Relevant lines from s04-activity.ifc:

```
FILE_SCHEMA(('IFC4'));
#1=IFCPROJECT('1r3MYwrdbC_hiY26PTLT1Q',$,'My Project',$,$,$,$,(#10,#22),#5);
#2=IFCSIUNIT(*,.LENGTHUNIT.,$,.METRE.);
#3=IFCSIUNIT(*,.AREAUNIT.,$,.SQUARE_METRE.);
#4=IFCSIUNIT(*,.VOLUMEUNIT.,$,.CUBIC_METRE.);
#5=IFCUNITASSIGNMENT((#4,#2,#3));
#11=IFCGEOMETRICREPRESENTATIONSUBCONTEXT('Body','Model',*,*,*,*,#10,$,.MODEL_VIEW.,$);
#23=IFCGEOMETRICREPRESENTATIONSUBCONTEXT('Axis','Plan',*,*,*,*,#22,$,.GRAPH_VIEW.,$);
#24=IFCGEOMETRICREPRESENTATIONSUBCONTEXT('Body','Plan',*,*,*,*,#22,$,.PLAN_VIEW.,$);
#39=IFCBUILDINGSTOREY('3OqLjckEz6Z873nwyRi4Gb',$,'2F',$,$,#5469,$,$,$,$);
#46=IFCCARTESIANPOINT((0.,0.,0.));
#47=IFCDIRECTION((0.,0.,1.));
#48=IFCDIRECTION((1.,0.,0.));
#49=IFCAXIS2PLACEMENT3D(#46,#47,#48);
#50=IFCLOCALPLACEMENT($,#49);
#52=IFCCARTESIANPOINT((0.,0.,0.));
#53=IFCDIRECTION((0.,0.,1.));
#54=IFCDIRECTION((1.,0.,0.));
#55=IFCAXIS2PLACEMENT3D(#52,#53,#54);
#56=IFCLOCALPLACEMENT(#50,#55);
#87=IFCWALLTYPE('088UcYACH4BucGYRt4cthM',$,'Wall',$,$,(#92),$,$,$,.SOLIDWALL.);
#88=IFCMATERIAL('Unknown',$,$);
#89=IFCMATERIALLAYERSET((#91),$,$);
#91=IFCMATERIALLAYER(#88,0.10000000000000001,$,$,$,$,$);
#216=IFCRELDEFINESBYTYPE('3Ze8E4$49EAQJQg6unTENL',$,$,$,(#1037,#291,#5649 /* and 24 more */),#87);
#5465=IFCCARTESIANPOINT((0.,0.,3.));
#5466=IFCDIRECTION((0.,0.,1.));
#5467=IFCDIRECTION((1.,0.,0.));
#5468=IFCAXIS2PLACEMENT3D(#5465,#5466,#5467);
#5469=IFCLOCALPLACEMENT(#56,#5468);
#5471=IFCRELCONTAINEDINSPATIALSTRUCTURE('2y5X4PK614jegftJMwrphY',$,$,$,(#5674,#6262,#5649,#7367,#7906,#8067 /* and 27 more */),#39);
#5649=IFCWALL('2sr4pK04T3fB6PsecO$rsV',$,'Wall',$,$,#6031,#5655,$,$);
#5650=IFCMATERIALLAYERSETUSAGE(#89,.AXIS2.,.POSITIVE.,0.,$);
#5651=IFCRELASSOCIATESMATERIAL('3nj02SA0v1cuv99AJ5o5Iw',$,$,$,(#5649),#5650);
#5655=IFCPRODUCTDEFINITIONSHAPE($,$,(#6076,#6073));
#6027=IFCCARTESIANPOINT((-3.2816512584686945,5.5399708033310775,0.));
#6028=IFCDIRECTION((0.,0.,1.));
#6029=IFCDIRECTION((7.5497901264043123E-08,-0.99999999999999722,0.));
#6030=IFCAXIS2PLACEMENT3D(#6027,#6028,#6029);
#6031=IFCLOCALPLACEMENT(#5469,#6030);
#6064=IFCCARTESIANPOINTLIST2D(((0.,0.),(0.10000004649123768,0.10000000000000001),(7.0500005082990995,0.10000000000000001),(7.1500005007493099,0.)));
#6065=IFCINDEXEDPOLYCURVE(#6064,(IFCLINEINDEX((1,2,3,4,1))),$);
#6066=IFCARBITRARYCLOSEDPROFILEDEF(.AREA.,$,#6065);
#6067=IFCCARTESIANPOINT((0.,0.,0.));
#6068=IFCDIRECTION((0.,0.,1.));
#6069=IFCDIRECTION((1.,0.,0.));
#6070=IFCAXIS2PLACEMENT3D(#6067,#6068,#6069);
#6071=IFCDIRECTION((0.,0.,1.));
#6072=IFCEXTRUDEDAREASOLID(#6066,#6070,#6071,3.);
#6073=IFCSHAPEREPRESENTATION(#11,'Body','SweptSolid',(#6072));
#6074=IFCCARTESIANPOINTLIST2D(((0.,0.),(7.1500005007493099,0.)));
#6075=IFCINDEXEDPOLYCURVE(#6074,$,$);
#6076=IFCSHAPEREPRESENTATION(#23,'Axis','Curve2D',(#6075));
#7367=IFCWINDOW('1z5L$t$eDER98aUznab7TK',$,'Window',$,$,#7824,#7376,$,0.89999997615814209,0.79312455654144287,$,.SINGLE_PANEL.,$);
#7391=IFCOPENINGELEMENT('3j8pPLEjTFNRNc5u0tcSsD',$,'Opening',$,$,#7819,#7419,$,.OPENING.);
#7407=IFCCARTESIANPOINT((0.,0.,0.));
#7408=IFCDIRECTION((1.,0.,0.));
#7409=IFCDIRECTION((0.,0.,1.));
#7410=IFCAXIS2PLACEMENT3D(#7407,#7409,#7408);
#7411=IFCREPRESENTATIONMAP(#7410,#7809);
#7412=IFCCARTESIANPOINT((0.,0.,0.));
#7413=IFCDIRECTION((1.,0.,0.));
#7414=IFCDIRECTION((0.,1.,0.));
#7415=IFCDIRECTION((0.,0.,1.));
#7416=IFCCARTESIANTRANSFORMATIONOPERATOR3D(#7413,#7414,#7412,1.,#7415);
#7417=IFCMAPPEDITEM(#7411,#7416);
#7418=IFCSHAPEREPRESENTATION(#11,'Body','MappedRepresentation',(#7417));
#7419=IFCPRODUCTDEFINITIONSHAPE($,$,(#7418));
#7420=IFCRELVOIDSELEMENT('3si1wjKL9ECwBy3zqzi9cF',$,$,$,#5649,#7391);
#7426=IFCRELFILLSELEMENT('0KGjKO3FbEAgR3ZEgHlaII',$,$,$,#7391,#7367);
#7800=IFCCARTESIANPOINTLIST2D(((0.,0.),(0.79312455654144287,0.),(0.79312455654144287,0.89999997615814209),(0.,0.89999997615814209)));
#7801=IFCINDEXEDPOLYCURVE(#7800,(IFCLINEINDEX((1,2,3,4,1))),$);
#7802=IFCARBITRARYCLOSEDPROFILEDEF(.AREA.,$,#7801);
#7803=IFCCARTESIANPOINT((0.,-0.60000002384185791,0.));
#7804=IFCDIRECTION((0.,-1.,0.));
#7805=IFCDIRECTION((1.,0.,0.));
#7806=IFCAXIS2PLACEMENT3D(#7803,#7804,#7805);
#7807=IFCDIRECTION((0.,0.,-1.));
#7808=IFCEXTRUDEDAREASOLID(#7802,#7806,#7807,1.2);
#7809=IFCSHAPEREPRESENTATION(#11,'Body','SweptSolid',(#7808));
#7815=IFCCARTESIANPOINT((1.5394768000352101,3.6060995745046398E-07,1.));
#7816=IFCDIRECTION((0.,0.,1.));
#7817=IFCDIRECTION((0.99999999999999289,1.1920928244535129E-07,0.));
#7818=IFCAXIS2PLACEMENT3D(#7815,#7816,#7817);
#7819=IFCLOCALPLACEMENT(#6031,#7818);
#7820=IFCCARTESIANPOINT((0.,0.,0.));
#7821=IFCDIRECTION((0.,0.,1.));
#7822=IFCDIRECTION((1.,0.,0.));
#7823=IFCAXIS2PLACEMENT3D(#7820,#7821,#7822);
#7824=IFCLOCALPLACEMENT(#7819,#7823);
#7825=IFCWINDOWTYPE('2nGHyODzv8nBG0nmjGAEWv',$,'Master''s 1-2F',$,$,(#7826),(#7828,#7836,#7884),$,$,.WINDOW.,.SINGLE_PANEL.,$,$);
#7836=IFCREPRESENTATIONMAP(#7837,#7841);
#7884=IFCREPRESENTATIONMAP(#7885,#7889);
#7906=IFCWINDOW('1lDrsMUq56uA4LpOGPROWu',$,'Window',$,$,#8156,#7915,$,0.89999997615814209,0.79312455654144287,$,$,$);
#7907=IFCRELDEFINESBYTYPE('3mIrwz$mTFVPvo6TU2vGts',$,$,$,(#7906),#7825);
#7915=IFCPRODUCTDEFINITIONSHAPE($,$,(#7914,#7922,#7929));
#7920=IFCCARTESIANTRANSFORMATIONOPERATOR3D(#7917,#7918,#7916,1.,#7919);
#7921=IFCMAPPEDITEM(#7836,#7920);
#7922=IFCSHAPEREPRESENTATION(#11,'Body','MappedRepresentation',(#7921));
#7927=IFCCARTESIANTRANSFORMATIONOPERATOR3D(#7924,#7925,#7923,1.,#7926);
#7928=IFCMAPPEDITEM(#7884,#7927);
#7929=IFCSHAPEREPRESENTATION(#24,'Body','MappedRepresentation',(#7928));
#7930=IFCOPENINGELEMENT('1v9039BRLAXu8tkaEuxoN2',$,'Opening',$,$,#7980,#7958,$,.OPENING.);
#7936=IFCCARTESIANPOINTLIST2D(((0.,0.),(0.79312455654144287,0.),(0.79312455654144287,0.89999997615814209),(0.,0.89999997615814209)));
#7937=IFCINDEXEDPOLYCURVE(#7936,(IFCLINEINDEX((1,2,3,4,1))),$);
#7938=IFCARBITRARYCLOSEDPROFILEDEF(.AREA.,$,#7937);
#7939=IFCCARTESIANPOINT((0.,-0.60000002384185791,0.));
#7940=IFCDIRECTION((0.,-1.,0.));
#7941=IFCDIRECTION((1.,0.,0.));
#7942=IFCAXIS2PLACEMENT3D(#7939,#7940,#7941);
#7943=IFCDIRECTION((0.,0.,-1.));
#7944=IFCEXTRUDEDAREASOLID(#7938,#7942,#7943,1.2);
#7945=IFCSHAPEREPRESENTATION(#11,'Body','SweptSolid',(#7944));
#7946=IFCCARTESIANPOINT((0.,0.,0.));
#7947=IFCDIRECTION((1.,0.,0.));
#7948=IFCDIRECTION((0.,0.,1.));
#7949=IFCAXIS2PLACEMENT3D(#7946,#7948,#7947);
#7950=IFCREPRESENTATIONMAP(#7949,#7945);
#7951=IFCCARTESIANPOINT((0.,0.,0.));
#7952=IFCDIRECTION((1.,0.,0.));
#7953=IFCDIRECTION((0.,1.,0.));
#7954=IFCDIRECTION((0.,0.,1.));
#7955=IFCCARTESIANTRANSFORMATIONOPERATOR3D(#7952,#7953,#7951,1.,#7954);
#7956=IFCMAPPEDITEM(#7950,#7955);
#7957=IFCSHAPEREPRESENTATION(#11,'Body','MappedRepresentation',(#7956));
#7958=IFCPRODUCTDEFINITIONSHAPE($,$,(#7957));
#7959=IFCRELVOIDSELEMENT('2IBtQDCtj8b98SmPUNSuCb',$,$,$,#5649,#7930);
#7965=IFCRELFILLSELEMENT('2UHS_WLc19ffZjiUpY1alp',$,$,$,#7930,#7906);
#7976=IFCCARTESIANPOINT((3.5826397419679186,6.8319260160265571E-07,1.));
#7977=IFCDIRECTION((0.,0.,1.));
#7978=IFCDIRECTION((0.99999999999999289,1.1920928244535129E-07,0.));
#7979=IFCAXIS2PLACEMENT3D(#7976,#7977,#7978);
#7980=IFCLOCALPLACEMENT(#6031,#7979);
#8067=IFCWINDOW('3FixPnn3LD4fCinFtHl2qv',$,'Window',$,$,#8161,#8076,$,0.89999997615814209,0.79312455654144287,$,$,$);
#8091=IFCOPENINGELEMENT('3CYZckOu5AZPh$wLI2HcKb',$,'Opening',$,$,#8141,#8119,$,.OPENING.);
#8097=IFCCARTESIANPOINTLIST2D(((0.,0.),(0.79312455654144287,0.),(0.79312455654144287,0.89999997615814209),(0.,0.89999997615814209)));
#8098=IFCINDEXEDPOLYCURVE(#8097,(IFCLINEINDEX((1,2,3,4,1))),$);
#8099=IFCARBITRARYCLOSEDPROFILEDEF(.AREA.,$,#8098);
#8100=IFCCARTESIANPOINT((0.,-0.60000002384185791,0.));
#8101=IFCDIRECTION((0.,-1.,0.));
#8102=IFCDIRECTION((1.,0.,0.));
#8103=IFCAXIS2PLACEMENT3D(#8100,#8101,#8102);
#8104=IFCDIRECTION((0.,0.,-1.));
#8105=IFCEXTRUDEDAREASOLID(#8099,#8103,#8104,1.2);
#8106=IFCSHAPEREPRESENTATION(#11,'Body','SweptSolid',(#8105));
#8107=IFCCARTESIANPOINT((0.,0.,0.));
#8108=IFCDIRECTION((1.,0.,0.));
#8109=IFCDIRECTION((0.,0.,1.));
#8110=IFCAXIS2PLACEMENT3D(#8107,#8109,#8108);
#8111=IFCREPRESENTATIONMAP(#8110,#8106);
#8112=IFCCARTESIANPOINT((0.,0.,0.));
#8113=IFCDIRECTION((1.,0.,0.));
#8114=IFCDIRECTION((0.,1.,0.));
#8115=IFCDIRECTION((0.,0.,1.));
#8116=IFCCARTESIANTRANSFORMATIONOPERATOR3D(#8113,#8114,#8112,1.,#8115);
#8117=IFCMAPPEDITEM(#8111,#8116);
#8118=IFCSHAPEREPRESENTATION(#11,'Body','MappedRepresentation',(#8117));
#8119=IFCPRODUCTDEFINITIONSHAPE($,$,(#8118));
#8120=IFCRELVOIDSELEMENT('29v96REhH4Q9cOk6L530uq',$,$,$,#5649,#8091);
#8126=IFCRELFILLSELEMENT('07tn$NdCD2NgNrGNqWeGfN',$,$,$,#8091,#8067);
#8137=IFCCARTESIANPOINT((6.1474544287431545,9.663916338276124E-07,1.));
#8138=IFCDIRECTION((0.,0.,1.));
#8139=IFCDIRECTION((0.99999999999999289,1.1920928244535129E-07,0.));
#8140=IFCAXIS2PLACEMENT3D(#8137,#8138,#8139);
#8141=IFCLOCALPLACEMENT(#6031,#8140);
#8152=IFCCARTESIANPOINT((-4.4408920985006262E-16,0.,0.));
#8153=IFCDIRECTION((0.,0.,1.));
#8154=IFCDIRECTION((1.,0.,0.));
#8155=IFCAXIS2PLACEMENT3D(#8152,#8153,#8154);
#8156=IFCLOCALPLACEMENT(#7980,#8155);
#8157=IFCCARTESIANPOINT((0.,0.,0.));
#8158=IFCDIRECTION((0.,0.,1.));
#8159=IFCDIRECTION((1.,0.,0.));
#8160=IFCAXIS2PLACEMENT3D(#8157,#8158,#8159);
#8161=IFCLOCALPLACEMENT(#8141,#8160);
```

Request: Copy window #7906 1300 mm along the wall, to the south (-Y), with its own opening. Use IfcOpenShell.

```python
import ifcopenshell
import ifcopenshell.api.feature
import ifcopenshell.api.geometry
import ifcopenshell.api.root
import ifcopenshell.geom
import ifcopenshell.util.element
import ifcopenshell.util.placement
import ifcopenshell.util.shape
import ifcopenshell.util.unit

model = ifcopenshell.open("s04-activity.ifc")
unit_scale = ifcopenshell.util.unit.calculate_unit_scale(model)
settings = ifcopenshell.geom.settings()


def volume(element):
    """Net volume in cubic metres, openings subtracted."""
    shape = ifcopenshell.geom.create_shape(settings, element)
    return ifcopenshell.util.shape.get_volume(shape.geometry)


window = model.by_id(7906)
opening = window.FillsVoids[0].RelatingOpeningElement
wall = opening.VoidsElements[0].RelatingBuildingElement
before = volume(wall)
shift = ifcopenshell.util.placement.get_local_placement(wall.ObjectPlacement)[:3, 0] * 1.3 / unit_scale

# copy_class copies the void relationship, type, container and properties, but no geometry.
new_opening = ifcopenshell.api.root.copy_class(model, product=opening)
new_opening.Representation = ifcopenshell.util.element.copy_deep(
    model, opening.Representation, exclude=["IfcGeometricRepresentationContext", "IfcRepresentationMap"]
)
new_window = ifcopenshell.api.root.copy_class(model, product=window)
new_window.Representation = ifcopenshell.util.element.copy_deep(
    model, window.Representation, exclude=["IfcGeometricRepresentationContext", "IfcRepresentationMap"]
)
ifcopenshell.api.feature.add_filling(model, opening=new_opening, element=new_window)

for old, new in ((opening, new_opening), (window, new_window)):
    matrix = ifcopenshell.util.placement.get_local_placement(old.ObjectPlacement)
    matrix[:3, 3] += shift
    ifcopenshell.api.geometry.edit_object_placement(model, product=new, matrix=matrix, is_si=False)

after = volume(wall)

print(f"wall volume {before:.3f} -> {after:.3f} m3")

model.write("s04-activity_v2.ifc")
```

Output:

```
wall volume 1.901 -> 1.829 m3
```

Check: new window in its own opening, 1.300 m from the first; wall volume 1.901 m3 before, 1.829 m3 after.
